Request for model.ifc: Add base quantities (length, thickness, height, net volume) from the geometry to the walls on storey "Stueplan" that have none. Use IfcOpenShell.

First a look at what the model holds.

```python
import ifcopenshell
import ifcopenshell.util.element
import ifcopenshell.util.unit

model = ifcopenshell.open("model.ifc")
print(model.schema)
for unit_type in ("LENGTHUNIT", "AREAUNIT", "VOLUMEUNIT"):
    print(unit_type, ifcopenshell.util.unit.calculate_unit_scale(model, unit_type))
storey = next(s for s in model.by_type("IfcBuildingStorey") if s.Name == "Stueplan")
walls = [e for e in ifcopenshell.util.element.get_decomposition(storey) if e.is_a("IfcWall")]
for e in sorted(walls, key=lambda e: e.id()):
    print(e.id(), e.is_a(), e.Name, list(ifcopenshell.util.element.get_psets(e, qtos_only=True)), sep=" | ")
```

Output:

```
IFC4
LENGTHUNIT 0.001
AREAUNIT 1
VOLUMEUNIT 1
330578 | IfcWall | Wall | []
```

```python
import ifcopenshell
import ifcopenshell.api.pset
import ifcopenshell.geom
import ifcopenshell.util.element
import ifcopenshell.util.shape
import ifcopenshell.util.unit

model = ifcopenshell.open("model.ifc")
unit_scale = ifcopenshell.util.unit.calculate_unit_scale(model)
volume_scale = ifcopenshell.util.unit.calculate_unit_scale(model, "VOLUMEUNIT")
settings = ifcopenshell.geom.settings()

storey = next(s for s in model.by_type("IfcBuildingStorey") if s.Name == "Stueplan")
walls = [e for e in ifcopenshell.util.element.get_decomposition(storey) if e.is_a("IfcWall")]

for e in sorted(walls, key=lambda e: e.id()):
    if ifcopenshell.util.element.get_psets(e, qtos_only=True, should_inherit=False):
        continue
    # Geometry comes back in metres, in the element's own axes.
    shape = ifcopenshell.geom.create_shape(settings, e)
    values = {
        "Length": ifcopenshell.util.shape.get_x(shape.geometry) / unit_scale,
        "Width": ifcopenshell.util.shape.get_y(shape.geometry) / unit_scale,
        "Height": ifcopenshell.util.shape.get_z(shape.geometry) / unit_scale,
        "NetVolume": ifcopenshell.util.shape.get_volume(shape.geometry) / volume_scale,
    }
    qto = ifcopenshell.api.pset.add_qto(model, product=e, name="Qto_WallBaseQuantities")
    ifcopenshell.api.pset.edit_qto(model, qto=qto, properties=values)
    print(e.id(), {k: round(v, 3) for k, v in values.items()})

model.write("model_edited.ifc")
```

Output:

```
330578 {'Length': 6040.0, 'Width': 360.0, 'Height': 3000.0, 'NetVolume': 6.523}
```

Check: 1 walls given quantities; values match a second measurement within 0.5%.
